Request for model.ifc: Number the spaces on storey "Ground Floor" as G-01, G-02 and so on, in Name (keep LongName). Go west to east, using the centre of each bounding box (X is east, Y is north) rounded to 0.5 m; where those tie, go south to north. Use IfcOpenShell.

First a look at what the model holds.

```python
import ifcopenshell
import ifcopenshell.util.element
import ifcopenshell.util.placement

model = ifcopenshell.open("model.ifc")
print(model.schema)
storey = next(s for s in model.by_type("IfcBuildingStorey") if s.Name == "Ground Floor")
spaces = [e for e in ifcopenshell.util.element.get_decomposition(storey) if e.is_a("IfcSpace")]
for e in sorted(spaces, key=lambda e: e.id()):
    origin = ifcopenshell.util.placement.get_local_placement(e.ObjectPlacement)[:3, 3]
    print(e.id(), e.Name, e.LongName, origin.round(2) + 0.0, sep=" | ")
```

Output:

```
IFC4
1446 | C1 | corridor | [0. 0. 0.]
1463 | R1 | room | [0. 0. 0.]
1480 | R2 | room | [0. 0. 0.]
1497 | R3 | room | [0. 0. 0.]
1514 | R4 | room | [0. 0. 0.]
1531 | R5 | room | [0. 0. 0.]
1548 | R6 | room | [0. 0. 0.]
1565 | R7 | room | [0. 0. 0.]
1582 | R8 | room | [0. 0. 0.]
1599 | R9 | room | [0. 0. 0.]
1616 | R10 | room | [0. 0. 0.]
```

```python
import ifcopenshell
import ifcopenshell.geom
import ifcopenshell.util.element
import ifcopenshell.util.shape

model = ifcopenshell.open("model.ifc")
settings = ifcopenshell.geom.settings()
settings.set("use-world-coords", True)


def centre(element):
    shape = ifcopenshell.geom.create_shape(settings, element)
    return ifcopenshell.util.shape.get_bbox_centroid(shape.geometry)


storey = next(s for s in model.by_type("IfcBuildingStorey") if s.Name == "Ground Floor")
spaces = [e for e in ifcopenshell.util.element.get_decomposition(storey) if e.is_a("IfcSpace")]

# Insertion points can sit at a corner or the storey origin, so sort by the geometry (in metres).
centres = {e: centre(e) for e in spaces}
spaces.sort(key=lambda e: (round(centres[e][0] / 0.5), centres[e][1]))

for i, e in enumerate(spaces, start=1):
    number = f"G-{i:02d}"
    e.Name = number
    print(e.id(), number)

model.write("model_updated.ifc")
```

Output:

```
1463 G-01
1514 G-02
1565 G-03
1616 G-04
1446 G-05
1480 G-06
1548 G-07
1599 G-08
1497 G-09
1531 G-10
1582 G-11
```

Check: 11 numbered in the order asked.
